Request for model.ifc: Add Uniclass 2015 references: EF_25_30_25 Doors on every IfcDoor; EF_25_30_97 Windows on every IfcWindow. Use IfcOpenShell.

First a look at what the model holds.

```python
import ifcopenshell

model = ifcopenshell.open("model.ifc")
print(model.schema)
print("classifications:", [c.Name for c in model.by_type("IfcClassification")])
for ifc_class in ("IfcDoor", "IfcRoof", "IfcStair", "IfcWall", "IfcWindow"):
    print(ifc_class, len(model.by_type(ifc_class)))
```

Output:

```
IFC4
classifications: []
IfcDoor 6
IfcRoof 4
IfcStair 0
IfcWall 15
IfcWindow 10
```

```python
import ifcopenshell
import ifcopenshell.api.classification

model = ifcopenshell.open("model.ifc")

system = ifcopenshell.api.classification.add_classification(model, classification="Uniclass 2015")

codes = {
    "IfcDoor": ("EF_25_30_25", "Doors"),
    "IfcWindow": ("EF_25_30_97", "Windows"),
}
for ifc_class, (code, name) in codes.items():
    products = model.by_type(ifc_class)
    ifcopenshell.api.classification.add_reference(
        model, products=products, classification=system, identification=code, name=name
    )
    print(code, len(products))

model.write("model_rev.ifc")
```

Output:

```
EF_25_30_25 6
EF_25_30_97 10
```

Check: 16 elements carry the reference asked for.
